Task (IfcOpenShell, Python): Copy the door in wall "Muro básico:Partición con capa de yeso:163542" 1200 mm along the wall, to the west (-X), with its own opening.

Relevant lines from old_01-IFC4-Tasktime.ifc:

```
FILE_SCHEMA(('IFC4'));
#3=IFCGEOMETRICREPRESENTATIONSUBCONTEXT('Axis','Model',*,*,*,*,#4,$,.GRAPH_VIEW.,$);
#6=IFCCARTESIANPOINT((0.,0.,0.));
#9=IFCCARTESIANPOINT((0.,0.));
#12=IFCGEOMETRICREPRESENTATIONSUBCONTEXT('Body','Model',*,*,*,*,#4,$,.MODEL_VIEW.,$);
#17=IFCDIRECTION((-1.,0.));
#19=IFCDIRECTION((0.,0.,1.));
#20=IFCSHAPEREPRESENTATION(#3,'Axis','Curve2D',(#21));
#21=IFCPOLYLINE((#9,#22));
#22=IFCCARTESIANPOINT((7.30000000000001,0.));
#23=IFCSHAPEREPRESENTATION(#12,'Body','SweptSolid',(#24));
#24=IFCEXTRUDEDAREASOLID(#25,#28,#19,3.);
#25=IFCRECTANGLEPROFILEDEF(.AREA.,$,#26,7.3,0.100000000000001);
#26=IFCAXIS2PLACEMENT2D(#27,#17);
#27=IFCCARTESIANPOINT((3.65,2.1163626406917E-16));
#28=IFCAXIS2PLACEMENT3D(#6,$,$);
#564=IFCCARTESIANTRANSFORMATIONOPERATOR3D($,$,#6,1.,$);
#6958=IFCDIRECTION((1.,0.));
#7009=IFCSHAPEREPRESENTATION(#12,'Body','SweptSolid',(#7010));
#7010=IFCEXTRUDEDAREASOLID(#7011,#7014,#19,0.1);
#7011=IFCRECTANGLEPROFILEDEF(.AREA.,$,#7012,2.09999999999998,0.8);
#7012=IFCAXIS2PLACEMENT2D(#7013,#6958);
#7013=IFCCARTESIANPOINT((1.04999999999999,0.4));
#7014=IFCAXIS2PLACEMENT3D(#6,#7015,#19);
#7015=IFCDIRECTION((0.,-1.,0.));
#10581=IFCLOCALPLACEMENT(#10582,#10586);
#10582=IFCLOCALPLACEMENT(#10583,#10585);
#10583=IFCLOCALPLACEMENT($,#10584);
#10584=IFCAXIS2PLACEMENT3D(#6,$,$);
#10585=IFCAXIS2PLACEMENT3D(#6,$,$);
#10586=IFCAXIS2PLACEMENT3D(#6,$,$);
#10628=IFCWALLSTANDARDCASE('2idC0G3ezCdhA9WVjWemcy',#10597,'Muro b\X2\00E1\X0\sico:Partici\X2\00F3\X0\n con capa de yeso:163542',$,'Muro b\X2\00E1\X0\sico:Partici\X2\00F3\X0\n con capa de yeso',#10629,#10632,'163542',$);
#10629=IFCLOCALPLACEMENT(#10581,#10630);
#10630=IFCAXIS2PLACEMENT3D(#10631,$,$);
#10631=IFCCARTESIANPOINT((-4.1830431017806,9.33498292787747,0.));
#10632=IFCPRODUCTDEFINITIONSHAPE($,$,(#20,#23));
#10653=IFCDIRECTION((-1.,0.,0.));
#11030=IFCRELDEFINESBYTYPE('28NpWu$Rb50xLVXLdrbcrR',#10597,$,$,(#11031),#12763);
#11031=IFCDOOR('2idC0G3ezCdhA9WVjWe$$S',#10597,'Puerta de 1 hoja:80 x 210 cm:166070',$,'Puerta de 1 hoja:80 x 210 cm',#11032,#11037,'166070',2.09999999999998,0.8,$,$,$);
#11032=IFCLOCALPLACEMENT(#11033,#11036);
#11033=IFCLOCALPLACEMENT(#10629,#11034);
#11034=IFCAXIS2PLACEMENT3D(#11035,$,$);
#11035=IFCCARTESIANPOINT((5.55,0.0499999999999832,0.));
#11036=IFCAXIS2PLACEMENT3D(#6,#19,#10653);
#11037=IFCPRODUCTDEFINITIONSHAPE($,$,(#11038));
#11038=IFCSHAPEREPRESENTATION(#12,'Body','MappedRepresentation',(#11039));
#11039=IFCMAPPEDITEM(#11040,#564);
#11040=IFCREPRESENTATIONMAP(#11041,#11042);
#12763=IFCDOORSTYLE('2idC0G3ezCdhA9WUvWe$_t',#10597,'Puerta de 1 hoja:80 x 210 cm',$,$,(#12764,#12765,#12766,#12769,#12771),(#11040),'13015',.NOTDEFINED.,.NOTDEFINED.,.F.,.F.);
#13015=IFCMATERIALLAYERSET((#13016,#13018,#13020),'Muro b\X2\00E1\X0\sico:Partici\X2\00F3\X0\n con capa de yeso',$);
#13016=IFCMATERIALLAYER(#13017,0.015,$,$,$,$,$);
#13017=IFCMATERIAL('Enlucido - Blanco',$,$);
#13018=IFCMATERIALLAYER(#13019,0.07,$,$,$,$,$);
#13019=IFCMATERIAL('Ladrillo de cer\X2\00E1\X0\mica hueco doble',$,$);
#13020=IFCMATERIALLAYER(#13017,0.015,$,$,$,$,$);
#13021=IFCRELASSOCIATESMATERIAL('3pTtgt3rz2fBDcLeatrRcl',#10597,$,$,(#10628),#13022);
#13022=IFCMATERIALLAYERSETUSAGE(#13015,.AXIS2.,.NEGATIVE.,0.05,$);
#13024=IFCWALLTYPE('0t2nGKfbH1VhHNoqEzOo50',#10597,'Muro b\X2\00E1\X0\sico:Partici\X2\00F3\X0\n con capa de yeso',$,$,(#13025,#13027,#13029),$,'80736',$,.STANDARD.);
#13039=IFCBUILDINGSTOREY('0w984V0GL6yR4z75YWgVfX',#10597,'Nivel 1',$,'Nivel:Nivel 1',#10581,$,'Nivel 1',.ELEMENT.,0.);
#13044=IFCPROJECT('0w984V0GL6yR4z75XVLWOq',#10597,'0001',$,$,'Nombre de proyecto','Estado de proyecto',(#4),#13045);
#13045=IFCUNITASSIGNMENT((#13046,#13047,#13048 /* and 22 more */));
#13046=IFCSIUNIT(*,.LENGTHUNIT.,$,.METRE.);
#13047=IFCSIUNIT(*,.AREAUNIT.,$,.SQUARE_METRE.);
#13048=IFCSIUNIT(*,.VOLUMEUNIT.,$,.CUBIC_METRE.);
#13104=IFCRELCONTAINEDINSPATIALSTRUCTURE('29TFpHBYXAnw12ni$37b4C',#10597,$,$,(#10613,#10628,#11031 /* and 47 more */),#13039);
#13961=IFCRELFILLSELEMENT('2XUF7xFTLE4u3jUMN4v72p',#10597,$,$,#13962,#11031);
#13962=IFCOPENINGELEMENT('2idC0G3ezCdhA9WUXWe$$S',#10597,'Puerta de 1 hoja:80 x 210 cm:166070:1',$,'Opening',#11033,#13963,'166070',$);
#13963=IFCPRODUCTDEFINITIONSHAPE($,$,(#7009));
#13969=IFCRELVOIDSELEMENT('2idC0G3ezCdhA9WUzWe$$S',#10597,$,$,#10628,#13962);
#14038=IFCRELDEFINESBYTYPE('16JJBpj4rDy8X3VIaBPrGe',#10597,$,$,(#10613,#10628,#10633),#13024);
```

```python
import ifcopenshell
import ifcopenshell.api.feature
import ifcopenshell.api.geometry
import ifcopenshell.api.root
import ifcopenshell.geom
import ifcopenshell.util.element
import ifcopenshell.util.placement
import ifcopenshell.util.shape
import ifcopenshell.util.unit

model = ifcopenshell.open("old_01-IFC4-Tasktime.ifc")
unit_scale = ifcopenshell.util.unit.calculate_unit_scale(model)
settings = ifcopenshell.geom.settings()


def volume(element):
    """Net volume in cubic metres, openings subtracted."""
    shape = ifcopenshell.geom.create_shape(settings, element)
    return ifcopenshell.util.shape.get_volume(shape.geometry)


def reuse_history(source, copy):
    """copy_class also copies each property set's owner history, people and application; keep the originals."""
    for rel in copy.IsDefinedBy:
        if rel.is_a("IfcRelDefinesByProperties") and (history := rel.RelatingPropertyDefinition.OwnerHistory):
            rel.RelatingPropertyDefinition.OwnerHistory = source.OwnerHistory
            ifcopenshell.util.element.remove_deep2(model, history)


door = model.by_guid("2idC0G3ezCdhA9WVjWe$$S")
opening = door.FillsVoids[0].RelatingOpeningElement
wall = opening.VoidsElements[0].RelatingBuildingElement
before = volume(wall)
shift = ifcopenshell.util.placement.get_local_placement(wall.ObjectPlacement)[:3, 0] * -1.2 / unit_scale

# copy_class copies the void relationship, type, container and properties, but no geometry.
new_opening = ifcopenshell.api.root.copy_class(model, product=opening)
new_opening.Representation = ifcopenshell.util.element.copy_deep(
    model, opening.Representation, exclude=["IfcGeometricRepresentationContext", "IfcRepresentationMap"]
)
new_opening.Name = "Puerta de 1 hoja:80 x 210 cm"
new_opening.Tag = None
new_door = ifcopenshell.api.root.copy_class(model, product=door)
new_door.Representation = ifcopenshell.util.element.copy_deep(
    model, door.Representation, exclude=["IfcGeometricRepresentationContext", "IfcRepresentationMap"]
)
new_door.Name = "Puerta de 1 hoja:80 x 210 cm"
new_door.Tag = None
reuse_history(door, new_door)
ifcopenshell.api.feature.add_filling(model, opening=new_opening, element=new_door)

for old, new in ((opening, new_opening), (door, new_door)):
    matrix = ifcopenshell.util.placement.get_local_placement(old.ObjectPlacement)
    matrix[:3, 3] += shift
    ifcopenshell.api.geometry.edit_object_placement(model, product=new, matrix=matrix, is_si=False)

after = volume(wall)

print(f"wall volume {before:.3f} -> {after:.3f} m3")

model.write("old_01-IFC4-Tasktime_rev.ifc")
```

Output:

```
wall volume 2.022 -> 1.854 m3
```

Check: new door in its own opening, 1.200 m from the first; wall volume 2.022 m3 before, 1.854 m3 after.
